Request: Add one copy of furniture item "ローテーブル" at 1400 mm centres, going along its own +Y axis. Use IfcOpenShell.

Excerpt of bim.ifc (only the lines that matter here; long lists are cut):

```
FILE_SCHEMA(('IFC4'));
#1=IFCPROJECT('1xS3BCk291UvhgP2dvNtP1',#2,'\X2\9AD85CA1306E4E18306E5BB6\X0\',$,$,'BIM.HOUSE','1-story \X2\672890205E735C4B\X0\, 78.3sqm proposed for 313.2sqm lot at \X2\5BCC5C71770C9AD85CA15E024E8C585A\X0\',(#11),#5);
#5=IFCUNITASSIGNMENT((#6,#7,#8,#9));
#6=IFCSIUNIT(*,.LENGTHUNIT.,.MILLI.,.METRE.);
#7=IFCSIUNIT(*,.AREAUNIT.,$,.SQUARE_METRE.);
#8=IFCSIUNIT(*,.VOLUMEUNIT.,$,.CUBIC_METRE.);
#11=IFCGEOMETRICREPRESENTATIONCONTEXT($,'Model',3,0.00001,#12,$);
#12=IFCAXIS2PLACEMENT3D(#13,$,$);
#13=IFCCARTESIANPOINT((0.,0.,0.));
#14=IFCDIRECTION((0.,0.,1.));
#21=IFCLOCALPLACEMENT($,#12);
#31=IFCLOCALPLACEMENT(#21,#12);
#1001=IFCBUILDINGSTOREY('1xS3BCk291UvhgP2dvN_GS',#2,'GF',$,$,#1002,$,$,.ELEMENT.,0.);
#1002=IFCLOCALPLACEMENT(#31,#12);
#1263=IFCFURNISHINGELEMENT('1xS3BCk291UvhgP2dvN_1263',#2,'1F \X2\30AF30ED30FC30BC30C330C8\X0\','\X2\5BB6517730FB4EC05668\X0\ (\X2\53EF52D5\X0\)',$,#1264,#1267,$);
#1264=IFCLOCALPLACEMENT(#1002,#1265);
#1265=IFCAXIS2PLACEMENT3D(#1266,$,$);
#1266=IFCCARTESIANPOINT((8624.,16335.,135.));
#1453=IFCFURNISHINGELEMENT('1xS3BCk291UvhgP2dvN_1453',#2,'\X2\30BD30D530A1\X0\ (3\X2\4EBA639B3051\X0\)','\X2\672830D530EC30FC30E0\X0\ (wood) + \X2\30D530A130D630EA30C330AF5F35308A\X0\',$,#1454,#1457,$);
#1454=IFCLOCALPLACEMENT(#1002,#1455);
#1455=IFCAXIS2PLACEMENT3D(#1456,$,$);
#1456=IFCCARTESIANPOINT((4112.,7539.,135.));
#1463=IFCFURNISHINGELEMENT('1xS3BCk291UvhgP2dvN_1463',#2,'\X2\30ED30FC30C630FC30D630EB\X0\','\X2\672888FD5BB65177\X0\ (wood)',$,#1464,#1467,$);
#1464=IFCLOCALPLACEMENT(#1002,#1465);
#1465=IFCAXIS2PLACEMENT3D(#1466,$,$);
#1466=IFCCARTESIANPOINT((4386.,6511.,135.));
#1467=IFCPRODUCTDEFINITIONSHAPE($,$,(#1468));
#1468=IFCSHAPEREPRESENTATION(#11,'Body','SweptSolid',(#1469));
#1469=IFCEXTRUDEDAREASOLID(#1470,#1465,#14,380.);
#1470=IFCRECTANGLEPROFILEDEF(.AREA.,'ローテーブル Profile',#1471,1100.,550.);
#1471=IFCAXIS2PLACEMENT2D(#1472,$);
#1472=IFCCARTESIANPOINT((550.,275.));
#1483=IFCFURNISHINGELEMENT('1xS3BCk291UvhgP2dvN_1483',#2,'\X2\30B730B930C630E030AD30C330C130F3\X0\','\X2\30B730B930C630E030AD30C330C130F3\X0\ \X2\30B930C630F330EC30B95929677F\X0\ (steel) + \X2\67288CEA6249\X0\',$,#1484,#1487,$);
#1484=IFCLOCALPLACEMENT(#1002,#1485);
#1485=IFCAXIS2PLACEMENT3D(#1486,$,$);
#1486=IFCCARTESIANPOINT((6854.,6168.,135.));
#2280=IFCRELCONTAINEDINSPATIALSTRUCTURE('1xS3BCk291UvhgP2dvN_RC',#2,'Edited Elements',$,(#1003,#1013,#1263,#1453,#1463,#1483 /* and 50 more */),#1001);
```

```python
import ifcopenshell
import ifcopenshell.api.geometry
import ifcopenshell.api.root
import ifcopenshell.util.element
import ifcopenshell.util.placement
import ifcopenshell.util.unit

model = ifcopenshell.open("bim.ifc")
unit_scale = ifcopenshell.util.unit.calculate_unit_scale(model)


def reuse_history(source, copy):
    """copy_class also copies each property set's owner history, people and application; keep the originals."""
    for rel in copy.IsDefinedBy:
        if rel.is_a("IfcRelDefinesByProperties") and (history := rel.RelatingPropertyDefinition.OwnerHistory):
            rel.RelatingPropertyDefinition.OwnerHistory = source.OwnerHistory
            ifcopenshell.util.element.remove_deep2(model, history)


source = model.by_guid("1xS3BCk291UvhgP2dvN_1463")
base = ifcopenshell.util.placement.get_local_placement(source.ObjectPlacement)
step = base[:3, 1] * 1.4 / unit_scale

for i in range(1, 2):
    copy = ifcopenshell.api.root.copy_class(model, product=source)
    copy.Representation = ifcopenshell.util.element.copy_deep(
        model, source.Representation, exclude=["IfcGeometricRepresentationContext", "IfcRepresentationMap"]
    )
    reuse_history(source, copy)
    matrix = base.copy()
    matrix[:3, 3] += i * step
    print("added at", matrix[:3, 3].round(3) + 0.0)
    ifcopenshell.api.geometry.edit_object_placement(model, product=copy, matrix=matrix, is_si=False)

model.write("bim-out.ifc")
```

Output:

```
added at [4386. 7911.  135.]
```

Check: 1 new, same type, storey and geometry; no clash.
